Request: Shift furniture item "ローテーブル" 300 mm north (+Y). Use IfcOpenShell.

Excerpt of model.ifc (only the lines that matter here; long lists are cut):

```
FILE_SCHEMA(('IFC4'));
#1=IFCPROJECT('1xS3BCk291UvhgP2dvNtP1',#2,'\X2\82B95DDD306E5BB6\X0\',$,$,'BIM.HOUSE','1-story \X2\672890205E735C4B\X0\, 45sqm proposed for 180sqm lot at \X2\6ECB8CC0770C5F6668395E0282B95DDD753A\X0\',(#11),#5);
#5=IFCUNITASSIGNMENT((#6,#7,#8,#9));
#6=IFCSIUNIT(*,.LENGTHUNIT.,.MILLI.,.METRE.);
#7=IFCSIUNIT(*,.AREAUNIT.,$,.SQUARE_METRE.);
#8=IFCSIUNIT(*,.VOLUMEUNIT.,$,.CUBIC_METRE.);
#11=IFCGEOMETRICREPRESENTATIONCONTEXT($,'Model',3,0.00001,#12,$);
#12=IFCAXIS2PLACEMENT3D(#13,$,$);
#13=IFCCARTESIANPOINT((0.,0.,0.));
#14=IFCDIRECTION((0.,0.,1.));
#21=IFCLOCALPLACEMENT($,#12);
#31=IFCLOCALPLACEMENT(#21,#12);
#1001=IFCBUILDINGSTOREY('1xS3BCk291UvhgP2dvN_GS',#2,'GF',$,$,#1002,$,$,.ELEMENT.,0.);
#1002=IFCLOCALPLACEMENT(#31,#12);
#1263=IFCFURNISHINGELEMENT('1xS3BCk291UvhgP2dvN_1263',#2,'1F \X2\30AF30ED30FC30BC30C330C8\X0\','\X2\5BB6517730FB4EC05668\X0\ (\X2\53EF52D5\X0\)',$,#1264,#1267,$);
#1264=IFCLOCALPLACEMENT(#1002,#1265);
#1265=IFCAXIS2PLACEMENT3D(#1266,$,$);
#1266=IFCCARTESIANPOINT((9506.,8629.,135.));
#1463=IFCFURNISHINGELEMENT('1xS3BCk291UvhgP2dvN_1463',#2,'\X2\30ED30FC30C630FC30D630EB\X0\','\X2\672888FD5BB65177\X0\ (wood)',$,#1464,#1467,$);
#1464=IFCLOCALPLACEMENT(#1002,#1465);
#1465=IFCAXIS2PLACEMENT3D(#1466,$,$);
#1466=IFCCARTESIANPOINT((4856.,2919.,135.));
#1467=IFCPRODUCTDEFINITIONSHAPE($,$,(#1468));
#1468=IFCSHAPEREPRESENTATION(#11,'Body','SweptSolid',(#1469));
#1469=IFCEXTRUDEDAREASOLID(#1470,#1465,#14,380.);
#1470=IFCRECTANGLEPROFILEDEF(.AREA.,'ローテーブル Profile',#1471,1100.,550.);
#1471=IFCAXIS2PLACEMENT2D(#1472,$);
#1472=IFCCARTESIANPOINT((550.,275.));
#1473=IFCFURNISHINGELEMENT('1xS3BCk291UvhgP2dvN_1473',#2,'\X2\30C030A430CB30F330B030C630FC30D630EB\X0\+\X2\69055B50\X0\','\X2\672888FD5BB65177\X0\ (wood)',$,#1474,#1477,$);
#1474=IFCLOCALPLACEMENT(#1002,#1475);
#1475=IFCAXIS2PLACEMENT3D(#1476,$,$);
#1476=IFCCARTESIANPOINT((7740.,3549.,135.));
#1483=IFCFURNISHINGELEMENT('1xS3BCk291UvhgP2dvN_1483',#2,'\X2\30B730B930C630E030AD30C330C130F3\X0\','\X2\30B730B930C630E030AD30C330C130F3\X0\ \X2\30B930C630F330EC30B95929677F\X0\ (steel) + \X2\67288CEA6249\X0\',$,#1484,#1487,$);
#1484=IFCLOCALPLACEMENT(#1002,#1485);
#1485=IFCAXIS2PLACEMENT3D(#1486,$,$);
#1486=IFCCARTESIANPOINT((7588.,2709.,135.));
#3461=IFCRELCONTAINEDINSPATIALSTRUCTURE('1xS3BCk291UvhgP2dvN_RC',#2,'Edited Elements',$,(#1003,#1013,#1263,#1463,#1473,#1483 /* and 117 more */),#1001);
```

```python
import ifcopenshell
import ifcopenshell.api.geometry
import ifcopenshell.util.placement

model = ifcopenshell.open("model.ifc")

item = model.by_guid("1xS3BCk291UvhgP2dvN_1463")
matrix = ifcopenshell.util.placement.get_local_placement(item.ObjectPlacement)
matrix[1, 3] += 300.0
ifcopenshell.api.geometry.edit_object_placement(model, product=item, matrix=matrix, is_si=False)

print(ifcopenshell.util.placement.get_local_placement(item.ObjectPlacement).round(3) + 0.0)

model.write("model-out.ifc")
```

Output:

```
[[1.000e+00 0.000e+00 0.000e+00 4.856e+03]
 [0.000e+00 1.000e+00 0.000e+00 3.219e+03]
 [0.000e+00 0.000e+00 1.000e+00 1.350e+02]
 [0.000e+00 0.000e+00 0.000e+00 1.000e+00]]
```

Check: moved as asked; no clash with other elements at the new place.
